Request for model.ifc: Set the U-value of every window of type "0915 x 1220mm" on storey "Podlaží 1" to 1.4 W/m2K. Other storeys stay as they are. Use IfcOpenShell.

First a look at what the model holds.

```python
import ifcopenshell
import ifcopenshell.util.element

model = ifcopenshell.open("model.ifc")
print(model.schema)
storey = next(s for s in model.by_type("IfcBuildingStorey") if s.Name == "Podlaží 1")
windows = [e for e in ifcopenshell.util.element.get_decomposition(storey) if e.is_a("IfcWindow")]
seen = {}
for e in windows:
    element_type = ifcopenshell.util.element.get_type(e)
    key = (element_type.Name if element_type != e and element_type else None, ifcopenshell.util.element.get_pset(e, "Pset_WindowCommon", "ThermalTransmittance"))
    seen[key] = seen.get(key, 0) + 1
for (name, value), count in sorted(seen.items(), key=str):
    print(count, "x", name, "|", value)
```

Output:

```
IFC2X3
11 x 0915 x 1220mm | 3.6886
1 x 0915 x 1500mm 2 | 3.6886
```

```python
import ifcopenshell
import ifcopenshell.api.pset
import ifcopenshell.util.element

model = ifcopenshell.open("model.ifc")

storey = next(s for s in model.by_type("IfcBuildingStorey") if s.Name == "Podlaží 1")
windows = [e for e in ifcopenshell.util.element.get_decomposition(storey) if e.is_a("IfcWindow")]

count = 0
for e in windows:
    element_type = ifcopenshell.util.element.get_type(e)
    if element_type in (None, e) or element_type.Name != "0915 x 1220mm":
        continue
    # add_pset returns the element's existing set when there is one.
    pset = ifcopenshell.api.pset.add_pset(model, product=e, name="Pset_WindowCommon")
    ifcopenshell.api.pset.edit_pset(model, pset=pset, properties={"ThermalTransmittance": 1.4})
    count += 1

print(count, "windows updated")

model.write("model_edited.ifc")
```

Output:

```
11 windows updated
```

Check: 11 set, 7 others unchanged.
